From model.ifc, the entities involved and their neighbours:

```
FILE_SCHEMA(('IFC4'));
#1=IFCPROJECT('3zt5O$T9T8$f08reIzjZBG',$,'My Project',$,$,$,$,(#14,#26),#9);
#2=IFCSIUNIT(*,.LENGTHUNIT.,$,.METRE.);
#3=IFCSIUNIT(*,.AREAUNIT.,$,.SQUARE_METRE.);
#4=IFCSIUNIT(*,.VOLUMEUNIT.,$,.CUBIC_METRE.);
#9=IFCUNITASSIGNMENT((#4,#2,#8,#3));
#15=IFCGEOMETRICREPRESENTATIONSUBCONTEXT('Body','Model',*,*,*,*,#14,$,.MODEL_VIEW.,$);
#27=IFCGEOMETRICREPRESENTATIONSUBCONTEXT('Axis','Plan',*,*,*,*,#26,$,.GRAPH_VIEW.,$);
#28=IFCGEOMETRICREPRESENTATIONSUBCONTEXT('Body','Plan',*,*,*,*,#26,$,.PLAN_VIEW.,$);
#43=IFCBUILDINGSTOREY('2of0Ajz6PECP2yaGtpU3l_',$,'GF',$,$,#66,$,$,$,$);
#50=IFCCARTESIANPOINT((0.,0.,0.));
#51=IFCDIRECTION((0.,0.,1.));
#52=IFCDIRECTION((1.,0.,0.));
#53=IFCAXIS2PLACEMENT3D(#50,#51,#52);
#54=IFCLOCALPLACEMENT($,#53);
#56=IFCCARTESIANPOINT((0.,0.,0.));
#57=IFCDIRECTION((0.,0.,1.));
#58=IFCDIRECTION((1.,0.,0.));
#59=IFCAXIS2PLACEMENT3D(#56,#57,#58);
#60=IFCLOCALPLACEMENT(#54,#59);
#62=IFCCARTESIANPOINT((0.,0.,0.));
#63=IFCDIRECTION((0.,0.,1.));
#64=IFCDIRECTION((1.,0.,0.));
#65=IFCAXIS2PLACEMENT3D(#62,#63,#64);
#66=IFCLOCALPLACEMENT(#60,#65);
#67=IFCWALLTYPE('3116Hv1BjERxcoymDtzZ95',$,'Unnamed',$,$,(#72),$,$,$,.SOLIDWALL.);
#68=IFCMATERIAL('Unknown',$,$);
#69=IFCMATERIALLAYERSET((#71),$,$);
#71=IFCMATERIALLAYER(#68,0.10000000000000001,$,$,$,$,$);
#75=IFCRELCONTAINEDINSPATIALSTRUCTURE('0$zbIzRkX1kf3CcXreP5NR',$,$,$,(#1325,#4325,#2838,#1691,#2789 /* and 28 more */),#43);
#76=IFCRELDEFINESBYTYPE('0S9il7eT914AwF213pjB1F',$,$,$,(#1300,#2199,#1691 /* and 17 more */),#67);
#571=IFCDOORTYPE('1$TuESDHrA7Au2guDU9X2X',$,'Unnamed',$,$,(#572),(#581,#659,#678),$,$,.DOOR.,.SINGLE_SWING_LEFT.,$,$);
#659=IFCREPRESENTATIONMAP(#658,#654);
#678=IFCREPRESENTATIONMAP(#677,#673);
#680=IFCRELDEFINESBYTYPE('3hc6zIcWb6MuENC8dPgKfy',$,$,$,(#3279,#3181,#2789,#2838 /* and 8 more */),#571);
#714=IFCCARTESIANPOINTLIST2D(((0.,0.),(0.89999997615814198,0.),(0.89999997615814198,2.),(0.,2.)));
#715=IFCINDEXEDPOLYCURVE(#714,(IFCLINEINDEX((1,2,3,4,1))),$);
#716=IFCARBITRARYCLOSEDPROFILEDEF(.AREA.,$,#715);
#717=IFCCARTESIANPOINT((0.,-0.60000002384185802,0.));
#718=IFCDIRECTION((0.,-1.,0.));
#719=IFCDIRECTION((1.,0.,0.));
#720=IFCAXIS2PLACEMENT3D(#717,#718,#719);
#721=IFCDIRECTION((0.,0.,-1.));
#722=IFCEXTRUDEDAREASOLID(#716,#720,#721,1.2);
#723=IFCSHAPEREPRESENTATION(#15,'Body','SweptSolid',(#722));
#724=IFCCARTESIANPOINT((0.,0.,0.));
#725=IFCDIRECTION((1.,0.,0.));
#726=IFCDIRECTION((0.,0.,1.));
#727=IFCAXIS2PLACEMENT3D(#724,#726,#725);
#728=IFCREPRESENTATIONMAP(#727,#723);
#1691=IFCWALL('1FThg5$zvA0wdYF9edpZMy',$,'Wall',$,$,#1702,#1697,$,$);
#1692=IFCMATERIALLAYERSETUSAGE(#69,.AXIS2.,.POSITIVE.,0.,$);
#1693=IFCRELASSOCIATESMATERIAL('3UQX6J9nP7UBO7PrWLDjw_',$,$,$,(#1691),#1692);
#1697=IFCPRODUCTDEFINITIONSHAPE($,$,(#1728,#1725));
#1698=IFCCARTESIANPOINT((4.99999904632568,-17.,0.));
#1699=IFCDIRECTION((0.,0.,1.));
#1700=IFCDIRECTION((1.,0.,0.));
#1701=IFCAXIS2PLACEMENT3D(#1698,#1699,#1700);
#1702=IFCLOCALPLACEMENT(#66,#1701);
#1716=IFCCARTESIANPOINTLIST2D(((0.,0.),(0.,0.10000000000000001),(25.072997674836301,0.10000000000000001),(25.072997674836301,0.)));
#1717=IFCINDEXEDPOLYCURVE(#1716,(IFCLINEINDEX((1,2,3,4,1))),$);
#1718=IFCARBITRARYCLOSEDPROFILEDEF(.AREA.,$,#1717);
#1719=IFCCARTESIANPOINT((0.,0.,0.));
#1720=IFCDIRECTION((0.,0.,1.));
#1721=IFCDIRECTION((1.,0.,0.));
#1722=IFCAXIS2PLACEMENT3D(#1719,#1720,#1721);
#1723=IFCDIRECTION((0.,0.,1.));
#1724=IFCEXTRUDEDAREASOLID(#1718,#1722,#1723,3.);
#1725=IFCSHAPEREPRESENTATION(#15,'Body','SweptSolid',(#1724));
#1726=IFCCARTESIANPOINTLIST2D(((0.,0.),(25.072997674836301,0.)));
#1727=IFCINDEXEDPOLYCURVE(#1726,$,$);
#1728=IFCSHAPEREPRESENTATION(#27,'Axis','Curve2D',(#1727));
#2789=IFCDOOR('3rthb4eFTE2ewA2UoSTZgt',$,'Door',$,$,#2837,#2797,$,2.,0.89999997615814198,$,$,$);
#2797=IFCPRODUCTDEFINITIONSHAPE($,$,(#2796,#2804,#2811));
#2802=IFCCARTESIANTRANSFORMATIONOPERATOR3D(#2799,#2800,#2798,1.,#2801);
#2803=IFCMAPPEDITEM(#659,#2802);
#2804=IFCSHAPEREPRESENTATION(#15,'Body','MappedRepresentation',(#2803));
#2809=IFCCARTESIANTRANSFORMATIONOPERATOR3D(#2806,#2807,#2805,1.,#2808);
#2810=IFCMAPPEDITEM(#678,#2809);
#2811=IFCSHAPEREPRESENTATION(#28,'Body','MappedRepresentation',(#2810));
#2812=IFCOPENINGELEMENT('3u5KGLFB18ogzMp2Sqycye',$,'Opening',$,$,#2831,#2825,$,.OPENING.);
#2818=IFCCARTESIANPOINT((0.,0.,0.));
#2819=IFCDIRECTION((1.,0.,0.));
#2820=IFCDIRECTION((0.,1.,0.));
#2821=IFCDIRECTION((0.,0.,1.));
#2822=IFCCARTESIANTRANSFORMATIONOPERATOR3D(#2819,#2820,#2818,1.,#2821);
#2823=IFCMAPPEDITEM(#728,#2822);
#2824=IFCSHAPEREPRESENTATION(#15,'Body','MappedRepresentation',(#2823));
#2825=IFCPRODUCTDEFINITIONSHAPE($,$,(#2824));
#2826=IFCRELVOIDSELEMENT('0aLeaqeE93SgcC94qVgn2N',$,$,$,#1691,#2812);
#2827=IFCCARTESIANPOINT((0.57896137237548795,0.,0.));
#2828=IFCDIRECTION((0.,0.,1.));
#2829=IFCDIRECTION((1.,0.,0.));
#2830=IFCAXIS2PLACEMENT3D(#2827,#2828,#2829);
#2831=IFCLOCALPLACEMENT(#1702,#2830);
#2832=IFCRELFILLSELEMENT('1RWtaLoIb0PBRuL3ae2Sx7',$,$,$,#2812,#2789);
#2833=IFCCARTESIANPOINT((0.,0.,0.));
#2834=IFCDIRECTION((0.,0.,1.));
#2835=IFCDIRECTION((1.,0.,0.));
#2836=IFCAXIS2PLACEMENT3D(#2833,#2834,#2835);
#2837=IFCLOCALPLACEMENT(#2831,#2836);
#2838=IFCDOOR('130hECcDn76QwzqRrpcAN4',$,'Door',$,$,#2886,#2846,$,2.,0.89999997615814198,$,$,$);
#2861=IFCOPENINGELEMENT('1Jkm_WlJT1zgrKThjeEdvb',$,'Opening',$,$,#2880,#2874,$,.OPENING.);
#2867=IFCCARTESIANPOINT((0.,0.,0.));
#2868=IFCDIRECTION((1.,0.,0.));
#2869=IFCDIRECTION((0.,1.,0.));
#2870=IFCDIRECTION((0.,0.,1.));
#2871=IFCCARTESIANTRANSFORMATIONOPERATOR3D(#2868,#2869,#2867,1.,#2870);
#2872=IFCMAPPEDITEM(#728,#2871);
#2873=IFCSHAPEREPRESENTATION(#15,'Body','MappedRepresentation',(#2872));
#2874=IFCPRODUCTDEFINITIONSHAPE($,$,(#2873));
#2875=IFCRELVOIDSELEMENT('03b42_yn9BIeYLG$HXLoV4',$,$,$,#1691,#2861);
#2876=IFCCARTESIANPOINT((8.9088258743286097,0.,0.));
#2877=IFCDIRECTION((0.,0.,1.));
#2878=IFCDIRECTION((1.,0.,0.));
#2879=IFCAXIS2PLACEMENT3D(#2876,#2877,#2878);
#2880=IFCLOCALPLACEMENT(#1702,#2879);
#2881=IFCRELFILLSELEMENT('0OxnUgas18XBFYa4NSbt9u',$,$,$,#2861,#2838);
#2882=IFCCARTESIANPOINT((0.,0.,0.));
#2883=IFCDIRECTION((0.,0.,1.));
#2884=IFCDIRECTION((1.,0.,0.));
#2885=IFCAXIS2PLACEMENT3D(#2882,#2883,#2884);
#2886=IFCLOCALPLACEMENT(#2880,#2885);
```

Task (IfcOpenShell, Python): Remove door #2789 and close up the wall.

```python
import ifcopenshell
import ifcopenshell.api.feature
import ifcopenshell.api.root
import ifcopenshell.geom
import ifcopenshell.util.shape

model = ifcopenshell.open("model.ifc")
settings = ifcopenshell.geom.settings()


def volume(element):
    """Net volume in cubic metres, openings subtracted."""
    shape = ifcopenshell.geom.create_shape(settings, element)
    return ifcopenshell.util.shape.get_volume(shape.geometry)


door = model.by_guid("3rthb4eFTE2ewA2UoSTZgt")
opening = door.FillsVoids[0].RelatingOpeningElement
wall = opening.VoidsElements[0].RelatingBuildingElement
before = volume(wall)

ifcopenshell.api.root.remove_product(model, product=door)
ifcopenshell.api.feature.remove_feature(model, feature=opening)

after = volume(wall)

print(f"wall volume {before:.3f} -> {after:.3f} m3")

model.write("model_updated.ifc")
```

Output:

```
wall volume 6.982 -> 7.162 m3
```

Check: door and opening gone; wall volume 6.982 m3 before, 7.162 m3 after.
